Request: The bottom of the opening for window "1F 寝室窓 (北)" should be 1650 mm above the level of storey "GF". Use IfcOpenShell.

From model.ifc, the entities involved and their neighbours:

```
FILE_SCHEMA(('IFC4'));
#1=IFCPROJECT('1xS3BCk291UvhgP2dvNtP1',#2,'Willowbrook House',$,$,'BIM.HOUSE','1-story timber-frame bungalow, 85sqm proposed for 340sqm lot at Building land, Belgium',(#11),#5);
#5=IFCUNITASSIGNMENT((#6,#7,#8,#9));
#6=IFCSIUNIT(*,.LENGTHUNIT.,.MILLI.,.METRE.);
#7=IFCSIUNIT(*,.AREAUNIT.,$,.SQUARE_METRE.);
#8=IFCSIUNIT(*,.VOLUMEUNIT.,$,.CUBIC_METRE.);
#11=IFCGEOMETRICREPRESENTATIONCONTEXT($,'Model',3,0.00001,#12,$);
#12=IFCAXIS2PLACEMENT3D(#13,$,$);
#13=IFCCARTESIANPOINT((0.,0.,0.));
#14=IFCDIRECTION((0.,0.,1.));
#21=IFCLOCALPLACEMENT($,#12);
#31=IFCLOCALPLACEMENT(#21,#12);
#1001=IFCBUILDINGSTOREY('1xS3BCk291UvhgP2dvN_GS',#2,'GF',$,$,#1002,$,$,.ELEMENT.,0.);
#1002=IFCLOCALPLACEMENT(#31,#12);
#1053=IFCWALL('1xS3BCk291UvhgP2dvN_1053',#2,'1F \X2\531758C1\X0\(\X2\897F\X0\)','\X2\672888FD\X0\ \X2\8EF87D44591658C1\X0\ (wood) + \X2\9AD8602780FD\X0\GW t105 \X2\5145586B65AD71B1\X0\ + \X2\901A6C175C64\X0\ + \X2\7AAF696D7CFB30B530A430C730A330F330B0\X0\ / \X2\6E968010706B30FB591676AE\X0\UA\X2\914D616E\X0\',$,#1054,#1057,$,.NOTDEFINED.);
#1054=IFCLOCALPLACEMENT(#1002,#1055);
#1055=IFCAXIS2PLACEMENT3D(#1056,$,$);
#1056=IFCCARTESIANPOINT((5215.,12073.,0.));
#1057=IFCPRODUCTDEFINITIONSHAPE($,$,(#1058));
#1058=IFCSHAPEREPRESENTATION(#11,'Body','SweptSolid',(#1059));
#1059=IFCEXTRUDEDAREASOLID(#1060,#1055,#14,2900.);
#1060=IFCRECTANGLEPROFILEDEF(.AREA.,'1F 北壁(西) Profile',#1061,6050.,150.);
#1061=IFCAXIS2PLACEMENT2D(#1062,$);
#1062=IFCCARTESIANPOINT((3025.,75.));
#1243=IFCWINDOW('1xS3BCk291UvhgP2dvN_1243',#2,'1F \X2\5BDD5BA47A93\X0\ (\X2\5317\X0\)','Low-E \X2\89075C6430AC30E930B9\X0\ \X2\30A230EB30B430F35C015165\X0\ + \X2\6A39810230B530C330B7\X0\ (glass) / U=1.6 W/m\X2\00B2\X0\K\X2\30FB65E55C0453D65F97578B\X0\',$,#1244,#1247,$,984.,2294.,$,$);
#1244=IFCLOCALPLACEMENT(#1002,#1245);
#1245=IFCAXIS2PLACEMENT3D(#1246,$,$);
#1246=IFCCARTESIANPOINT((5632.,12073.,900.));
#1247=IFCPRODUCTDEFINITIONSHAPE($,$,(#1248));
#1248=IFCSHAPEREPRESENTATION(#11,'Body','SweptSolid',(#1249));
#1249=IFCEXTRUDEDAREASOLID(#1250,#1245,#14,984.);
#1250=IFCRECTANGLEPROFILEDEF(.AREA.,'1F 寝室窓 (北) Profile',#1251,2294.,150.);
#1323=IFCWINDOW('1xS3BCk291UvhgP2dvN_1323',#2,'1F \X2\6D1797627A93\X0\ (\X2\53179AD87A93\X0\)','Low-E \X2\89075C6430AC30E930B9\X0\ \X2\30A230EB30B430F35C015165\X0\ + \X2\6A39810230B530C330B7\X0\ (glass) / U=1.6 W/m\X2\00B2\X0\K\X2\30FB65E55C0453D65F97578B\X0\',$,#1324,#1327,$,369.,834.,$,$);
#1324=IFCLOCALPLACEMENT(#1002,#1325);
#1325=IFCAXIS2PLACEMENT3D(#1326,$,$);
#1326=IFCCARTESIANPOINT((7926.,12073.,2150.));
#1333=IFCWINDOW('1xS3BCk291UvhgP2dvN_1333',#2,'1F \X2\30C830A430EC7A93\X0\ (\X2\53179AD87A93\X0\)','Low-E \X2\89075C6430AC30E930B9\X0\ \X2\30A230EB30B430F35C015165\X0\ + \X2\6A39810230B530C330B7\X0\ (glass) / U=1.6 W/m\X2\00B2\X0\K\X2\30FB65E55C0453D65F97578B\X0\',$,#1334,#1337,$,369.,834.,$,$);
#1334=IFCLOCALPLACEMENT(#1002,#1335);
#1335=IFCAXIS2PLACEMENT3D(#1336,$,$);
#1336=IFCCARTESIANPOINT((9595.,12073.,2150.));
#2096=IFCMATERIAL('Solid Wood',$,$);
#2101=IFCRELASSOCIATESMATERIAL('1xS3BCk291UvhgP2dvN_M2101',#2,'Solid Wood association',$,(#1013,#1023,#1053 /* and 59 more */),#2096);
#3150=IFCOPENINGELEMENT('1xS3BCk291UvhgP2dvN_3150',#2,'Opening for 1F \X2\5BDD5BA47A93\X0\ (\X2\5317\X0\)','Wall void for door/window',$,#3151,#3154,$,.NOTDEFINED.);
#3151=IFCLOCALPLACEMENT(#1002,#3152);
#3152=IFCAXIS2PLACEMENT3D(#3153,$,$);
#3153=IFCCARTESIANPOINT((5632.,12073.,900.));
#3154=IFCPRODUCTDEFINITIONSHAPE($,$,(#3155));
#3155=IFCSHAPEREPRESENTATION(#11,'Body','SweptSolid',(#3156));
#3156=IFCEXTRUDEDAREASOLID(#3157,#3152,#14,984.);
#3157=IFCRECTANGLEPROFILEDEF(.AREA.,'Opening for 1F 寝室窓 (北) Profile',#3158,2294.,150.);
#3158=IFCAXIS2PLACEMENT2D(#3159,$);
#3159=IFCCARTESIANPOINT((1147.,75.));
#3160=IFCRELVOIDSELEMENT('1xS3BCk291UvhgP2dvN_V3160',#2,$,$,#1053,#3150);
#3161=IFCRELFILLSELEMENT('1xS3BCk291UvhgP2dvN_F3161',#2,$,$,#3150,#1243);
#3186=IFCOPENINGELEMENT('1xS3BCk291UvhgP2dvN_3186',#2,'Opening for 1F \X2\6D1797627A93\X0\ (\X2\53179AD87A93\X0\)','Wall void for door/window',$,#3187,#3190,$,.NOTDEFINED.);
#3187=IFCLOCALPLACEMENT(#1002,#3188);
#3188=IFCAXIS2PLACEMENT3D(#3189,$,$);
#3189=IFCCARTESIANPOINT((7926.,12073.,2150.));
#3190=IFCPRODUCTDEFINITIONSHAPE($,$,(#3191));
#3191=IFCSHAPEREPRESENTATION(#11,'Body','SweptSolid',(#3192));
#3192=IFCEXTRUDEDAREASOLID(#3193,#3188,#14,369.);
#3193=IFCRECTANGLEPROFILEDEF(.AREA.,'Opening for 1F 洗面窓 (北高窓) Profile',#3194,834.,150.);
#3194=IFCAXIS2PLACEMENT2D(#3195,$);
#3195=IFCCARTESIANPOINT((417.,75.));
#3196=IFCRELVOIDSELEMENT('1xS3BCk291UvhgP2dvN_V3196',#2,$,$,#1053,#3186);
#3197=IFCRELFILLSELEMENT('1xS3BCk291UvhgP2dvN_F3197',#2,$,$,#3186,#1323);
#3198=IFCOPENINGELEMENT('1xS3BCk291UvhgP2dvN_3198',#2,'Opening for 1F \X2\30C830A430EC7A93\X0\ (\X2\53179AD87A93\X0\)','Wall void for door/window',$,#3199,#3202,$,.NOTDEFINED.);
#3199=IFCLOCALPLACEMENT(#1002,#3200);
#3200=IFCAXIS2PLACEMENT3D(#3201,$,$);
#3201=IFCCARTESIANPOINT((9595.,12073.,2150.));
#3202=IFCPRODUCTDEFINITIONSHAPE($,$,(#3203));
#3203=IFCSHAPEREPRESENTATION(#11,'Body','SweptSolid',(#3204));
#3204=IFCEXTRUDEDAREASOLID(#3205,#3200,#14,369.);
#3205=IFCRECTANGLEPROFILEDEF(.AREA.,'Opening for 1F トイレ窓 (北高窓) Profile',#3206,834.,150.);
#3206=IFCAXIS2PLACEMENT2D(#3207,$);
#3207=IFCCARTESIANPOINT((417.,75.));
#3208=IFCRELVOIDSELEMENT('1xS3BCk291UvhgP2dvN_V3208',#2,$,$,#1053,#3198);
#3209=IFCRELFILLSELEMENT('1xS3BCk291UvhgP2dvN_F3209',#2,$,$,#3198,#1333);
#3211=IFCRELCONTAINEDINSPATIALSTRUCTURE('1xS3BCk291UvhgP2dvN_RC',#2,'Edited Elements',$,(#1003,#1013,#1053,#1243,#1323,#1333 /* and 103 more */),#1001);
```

```python
import numpy as np
import ifcopenshell
import ifcopenshell.api.geometry
import ifcopenshell.geom
import ifcopenshell.util.element
import ifcopenshell.util.placement
import ifcopenshell.util.shape
import ifcopenshell.util.unit

model = ifcopenshell.open("model.ifc")
unit_scale = ifcopenshell.util.unit.calculate_unit_scale(model)

window = model.by_guid("1xS3BCk291UvhgP2dvN_1243")
opening = window.FillsVoids[0].RelatingOpeningElement
storey = ifcopenshell.util.element.get_container(window, ifc_class="IfcBuildingStorey")
level = ifcopenshell.util.placement.get_local_placement(storey.ObjectPlacement)[2, 3]

# The opening's origin need not be at the sill, so measure its lowest point.
shape = ifcopenshell.geom.create_shape(ifcopenshell.geom.settings(), opening)
bottom = ifcopenshell.util.shape.get_shape_bottom_elevation(shape, shape.geometry) / unit_scale
dz = level + 1.65 / unit_scale - bottom

shift = np.array([0.0, 0.0, dz])
# The window is not placed relative to its opening, so move both.
for product in (opening, window):
    matrix = ifcopenshell.util.placement.get_local_placement(product.ObjectPlacement)
    matrix[:3, 3] += shift
    ifcopenshell.api.geometry.edit_object_placement(model, product=product, matrix=matrix, is_si=False)

print(f"moved by {dz * unit_scale:+.3f} m")

model.write("model_rev.ifc")
```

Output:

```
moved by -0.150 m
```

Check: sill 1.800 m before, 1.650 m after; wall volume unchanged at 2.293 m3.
